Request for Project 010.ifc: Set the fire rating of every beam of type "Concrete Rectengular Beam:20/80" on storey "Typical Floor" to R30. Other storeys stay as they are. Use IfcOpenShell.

First a look at what the model holds.

```python
import ifcopenshell
import ifcopenshell.util.element

model = ifcopenshell.open("Project 010.ifc")
print(model.schema)
storey = next(s for s in model.by_type("IfcBuildingStorey") if s.Name == "Typical Floor")
beams = [e for e in ifcopenshell.util.element.get_decomposition(storey) if e.is_a("IfcBeam")]
seen = {}
for e in beams:
    element_type = ifcopenshell.util.element.get_type(e)
    key = (element_type.Name if element_type != e and element_type else None, ifcopenshell.util.element.get_pset(e, "Pset_BeamCommon", "FireRating"))
    seen[key] = seen.get(key, 0) + 1
for (name, value), count in sorted(seen.items(), key=str):
    print(count, "x", name, "|", value)
```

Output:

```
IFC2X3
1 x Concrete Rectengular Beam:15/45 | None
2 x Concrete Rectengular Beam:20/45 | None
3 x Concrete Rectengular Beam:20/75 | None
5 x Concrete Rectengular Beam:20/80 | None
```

```python
import ifcopenshell
import ifcopenshell.api.pset
import ifcopenshell.util.element

model = ifcopenshell.open("Project 010.ifc")

storey = next(s for s in model.by_type("IfcBuildingStorey") if s.Name == "Typical Floor")
beams = [e for e in ifcopenshell.util.element.get_decomposition(storey) if e.is_a("IfcBeam")]

count = 0
for e in beams:
    element_type = ifcopenshell.util.element.get_type(e)
    if element_type in (None, e) or element_type.Name != "Concrete Rectengular Beam:20/80":
        continue
    # add_pset returns the element's existing set when there is one.
    pset = ifcopenshell.api.pset.add_pset(model, product=e, name="Pset_BeamCommon")
    ifcopenshell.api.pset.edit_pset(model, pset=pset, properties={"FireRating": "R30"})
    count += 1

print(count, "beams updated")

model.write("Project 010_edited.ifc")
```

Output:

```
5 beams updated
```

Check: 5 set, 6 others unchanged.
